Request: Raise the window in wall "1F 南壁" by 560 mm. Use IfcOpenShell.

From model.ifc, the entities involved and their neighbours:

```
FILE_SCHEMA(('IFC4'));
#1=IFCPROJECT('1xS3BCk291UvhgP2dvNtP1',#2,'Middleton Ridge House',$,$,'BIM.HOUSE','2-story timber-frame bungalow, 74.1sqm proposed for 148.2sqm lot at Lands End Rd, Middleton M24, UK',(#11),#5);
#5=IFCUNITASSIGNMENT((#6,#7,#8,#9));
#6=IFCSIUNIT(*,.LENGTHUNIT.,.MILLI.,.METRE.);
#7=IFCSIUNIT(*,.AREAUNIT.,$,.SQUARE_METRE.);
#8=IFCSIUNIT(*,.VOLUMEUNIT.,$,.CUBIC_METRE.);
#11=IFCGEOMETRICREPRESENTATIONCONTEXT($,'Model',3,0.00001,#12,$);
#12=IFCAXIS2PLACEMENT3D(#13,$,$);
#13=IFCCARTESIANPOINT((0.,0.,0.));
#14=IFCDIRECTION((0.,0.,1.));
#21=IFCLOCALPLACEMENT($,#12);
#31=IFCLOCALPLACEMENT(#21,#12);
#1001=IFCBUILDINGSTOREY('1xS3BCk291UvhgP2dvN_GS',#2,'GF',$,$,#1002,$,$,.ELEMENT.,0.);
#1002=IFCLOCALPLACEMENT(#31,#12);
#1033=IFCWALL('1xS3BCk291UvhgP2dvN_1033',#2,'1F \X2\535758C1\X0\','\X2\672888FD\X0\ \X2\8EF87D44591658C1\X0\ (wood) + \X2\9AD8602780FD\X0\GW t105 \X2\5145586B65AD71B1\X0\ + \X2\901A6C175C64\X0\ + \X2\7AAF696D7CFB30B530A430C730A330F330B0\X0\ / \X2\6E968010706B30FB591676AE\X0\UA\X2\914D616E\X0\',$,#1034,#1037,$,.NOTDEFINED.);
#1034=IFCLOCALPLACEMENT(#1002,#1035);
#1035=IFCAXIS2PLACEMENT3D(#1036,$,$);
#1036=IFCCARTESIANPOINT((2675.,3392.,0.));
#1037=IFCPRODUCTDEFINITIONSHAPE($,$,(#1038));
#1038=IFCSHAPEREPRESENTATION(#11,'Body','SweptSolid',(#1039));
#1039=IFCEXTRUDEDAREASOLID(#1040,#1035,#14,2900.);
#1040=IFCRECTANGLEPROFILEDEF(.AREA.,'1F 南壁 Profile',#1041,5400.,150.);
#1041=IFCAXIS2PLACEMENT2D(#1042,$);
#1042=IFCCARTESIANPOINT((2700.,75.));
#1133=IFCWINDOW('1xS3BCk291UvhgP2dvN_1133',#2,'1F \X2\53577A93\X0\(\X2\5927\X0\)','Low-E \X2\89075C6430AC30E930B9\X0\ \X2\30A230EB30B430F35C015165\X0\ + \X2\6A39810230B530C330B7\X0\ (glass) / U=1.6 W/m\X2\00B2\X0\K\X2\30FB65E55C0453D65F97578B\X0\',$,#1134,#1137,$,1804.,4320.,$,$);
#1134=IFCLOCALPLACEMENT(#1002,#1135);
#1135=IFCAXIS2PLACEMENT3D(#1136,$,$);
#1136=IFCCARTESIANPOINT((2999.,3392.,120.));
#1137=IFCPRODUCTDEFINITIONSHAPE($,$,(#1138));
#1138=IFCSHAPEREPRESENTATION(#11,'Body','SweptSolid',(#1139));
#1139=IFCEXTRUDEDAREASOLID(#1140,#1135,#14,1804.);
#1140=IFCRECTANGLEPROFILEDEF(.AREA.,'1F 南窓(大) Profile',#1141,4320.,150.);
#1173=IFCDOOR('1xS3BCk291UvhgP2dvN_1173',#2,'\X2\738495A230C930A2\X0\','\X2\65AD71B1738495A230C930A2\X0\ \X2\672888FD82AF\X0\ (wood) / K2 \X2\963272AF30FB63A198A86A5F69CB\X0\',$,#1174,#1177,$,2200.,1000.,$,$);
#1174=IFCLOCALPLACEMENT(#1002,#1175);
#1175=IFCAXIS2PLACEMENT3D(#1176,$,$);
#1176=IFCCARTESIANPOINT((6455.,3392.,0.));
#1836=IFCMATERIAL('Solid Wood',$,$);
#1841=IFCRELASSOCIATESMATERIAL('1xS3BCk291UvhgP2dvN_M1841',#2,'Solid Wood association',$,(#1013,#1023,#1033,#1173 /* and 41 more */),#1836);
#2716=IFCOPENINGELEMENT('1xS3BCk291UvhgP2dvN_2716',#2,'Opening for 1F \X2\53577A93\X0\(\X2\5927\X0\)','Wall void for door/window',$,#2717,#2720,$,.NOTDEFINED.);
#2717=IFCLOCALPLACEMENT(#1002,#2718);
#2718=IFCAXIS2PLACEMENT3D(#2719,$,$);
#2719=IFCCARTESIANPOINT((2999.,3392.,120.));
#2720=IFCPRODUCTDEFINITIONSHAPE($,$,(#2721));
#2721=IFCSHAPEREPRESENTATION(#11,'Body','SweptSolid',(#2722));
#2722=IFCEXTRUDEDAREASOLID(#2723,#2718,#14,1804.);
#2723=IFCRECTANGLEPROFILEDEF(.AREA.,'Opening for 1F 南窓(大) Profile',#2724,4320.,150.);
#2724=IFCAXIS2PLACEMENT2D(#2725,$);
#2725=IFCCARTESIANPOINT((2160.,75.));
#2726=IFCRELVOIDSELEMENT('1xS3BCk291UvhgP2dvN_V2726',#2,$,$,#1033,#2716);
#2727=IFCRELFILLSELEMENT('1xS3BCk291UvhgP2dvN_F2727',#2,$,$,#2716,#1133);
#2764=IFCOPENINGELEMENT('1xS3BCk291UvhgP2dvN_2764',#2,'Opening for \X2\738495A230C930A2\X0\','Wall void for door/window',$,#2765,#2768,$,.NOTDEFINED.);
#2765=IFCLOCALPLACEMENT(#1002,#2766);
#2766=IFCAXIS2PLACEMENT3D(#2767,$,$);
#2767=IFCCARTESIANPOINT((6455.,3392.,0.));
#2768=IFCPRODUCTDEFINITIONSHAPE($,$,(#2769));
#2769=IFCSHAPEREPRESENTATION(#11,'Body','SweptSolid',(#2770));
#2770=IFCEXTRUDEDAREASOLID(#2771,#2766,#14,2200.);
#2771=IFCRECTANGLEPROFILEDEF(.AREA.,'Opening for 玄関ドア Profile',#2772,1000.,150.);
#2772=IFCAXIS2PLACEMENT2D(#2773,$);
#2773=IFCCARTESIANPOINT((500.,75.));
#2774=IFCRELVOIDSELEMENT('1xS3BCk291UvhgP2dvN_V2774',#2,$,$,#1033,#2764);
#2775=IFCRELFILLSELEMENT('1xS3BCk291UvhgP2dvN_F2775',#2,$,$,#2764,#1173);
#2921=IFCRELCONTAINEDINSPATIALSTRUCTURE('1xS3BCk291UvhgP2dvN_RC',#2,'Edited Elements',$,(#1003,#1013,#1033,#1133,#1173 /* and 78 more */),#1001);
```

```python
import numpy as np
import ifcopenshell
import ifcopenshell.api.geometry
import ifcopenshell.util.placement
import ifcopenshell.util.unit

model = ifcopenshell.open("model.ifc")
unit_scale = ifcopenshell.util.unit.calculate_unit_scale(model)

window = model.by_guid("1xS3BCk291UvhgP2dvN_1133")
opening = window.FillsVoids[0].RelatingOpeningElement
dz = 560.0

shift = np.array([0.0, 0.0, dz])
# The window is not placed relative to its opening, so move both.
for product in (opening, window):
    matrix = ifcopenshell.util.placement.get_local_placement(product.ObjectPlacement)
    matrix[:3, 3] += shift
    ifcopenshell.api.geometry.edit_object_placement(model, product=product, matrix=matrix, is_si=False)

print(f"moved by {dz * unit_scale:+.3f} m")

model.write("model_v2.ifc")
```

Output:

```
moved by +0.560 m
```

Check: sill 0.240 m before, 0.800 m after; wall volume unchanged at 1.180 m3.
